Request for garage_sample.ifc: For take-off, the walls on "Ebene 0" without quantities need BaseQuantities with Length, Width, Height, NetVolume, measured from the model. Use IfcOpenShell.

First a look at what the model holds.

```python
import ifcopenshell
import ifcopenshell.util.element
import ifcopenshell.util.unit

model = ifcopenshell.open("garage_sample.ifc")
print(model.schema)
for unit_type in ("LENGTHUNIT", "AREAUNIT", "VOLUMEUNIT"):
    print(unit_type, ifcopenshell.util.unit.calculate_unit_scale(model, unit_type))
storey = next(s for s in model.by_type("IfcBuildingStorey") if s.Name == "Ebene 0")
walls = [e for e in ifcopenshell.util.element.get_decomposition(storey) if e.is_a("IfcWall")]
for e in sorted(walls, key=lambda e: e.id()):
    print(e.id(), e.is_a(), e.Name, list(ifcopenshell.util.element.get_psets(e, qtos_only=True)), sep=" | ")
```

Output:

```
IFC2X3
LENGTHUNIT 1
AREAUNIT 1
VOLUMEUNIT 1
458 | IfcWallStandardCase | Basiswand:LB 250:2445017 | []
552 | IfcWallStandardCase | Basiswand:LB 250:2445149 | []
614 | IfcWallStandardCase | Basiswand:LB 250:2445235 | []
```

```python
import ifcopenshell
import ifcopenshell.api.pset
import ifcopenshell.geom
import ifcopenshell.util.element
import ifcopenshell.util.shape
import ifcopenshell.util.unit

model = ifcopenshell.open("garage_sample.ifc")
unit_scale = ifcopenshell.util.unit.calculate_unit_scale(model)
volume_scale = ifcopenshell.util.unit.calculate_unit_scale(model, "VOLUMEUNIT")
settings = ifcopenshell.geom.settings()

storey = next(s for s in model.by_type("IfcBuildingStorey") if s.Name == "Ebene 0")
walls = [e for e in ifcopenshell.util.element.get_decomposition(storey) if e.is_a("IfcWall")]

for e in sorted(walls, key=lambda e: e.id()):
    if ifcopenshell.util.element.get_psets(e, qtos_only=True, should_inherit=False):
        continue
    # Geometry comes back in metres, in the element's own axes.
    shape = ifcopenshell.geom.create_shape(settings, e)
    values = {
        "Length": ifcopenshell.util.shape.get_x(shape.geometry) / unit_scale,
        "Width": ifcopenshell.util.shape.get_y(shape.geometry) / unit_scale,
        "Height": ifcopenshell.util.shape.get_z(shape.geometry) / unit_scale,
        "NetVolume": ifcopenshell.util.shape.get_volume(shape.geometry) / volume_scale,
    }
    qto = ifcopenshell.api.pset.add_qto(model, product=e, name="BaseQuantities")
    ifcopenshell.api.pset.edit_qto(model, qto=qto, properties=values)
    print(e.id(), {k: round(v, 3) for k, v in values.items()})

model.write("garage_sample_v2.ifc")
```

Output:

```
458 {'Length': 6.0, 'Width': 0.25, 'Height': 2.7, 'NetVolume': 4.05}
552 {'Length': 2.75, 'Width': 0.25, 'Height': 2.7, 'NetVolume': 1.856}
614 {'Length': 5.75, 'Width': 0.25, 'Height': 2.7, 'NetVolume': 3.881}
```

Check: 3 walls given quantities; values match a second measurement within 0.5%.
